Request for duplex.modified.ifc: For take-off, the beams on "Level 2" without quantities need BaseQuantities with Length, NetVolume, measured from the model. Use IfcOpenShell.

First a look at what the model holds.

```python
import ifcopenshell
import ifcopenshell.util.element
import ifcopenshell.util.unit

model = ifcopenshell.open("duplex.modified.ifc")
print(model.schema)
for unit_type in ("LENGTHUNIT", "AREAUNIT", "VOLUMEUNIT"):
    print(unit_type, ifcopenshell.util.unit.calculate_unit_scale(model, unit_type))
storey = next(s for s in model.by_type("IfcBuildingStorey") if s.Name == "Level 2")
beams = [e for e in ifcopenshell.util.element.get_decomposition(storey) if e.is_a("IfcBeam")]
for e in sorted(beams, key=lambda e: e.id()):
    print(e.id(), e.is_a(), e.Name, list(ifcopenshell.util.element.get_psets(e, qtos_only=True)), sep=" | ")
```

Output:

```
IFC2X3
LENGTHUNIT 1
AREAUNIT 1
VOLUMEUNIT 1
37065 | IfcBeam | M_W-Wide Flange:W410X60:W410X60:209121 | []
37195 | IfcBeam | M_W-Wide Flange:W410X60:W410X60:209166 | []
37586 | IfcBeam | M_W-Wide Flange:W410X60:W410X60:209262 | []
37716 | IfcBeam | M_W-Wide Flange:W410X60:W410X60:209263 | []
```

```python
import ifcopenshell
import ifcopenshell.api.pset
import ifcopenshell.geom
import ifcopenshell.util.element
import ifcopenshell.util.shape
import ifcopenshell.util.unit

model = ifcopenshell.open("duplex.modified.ifc")
unit_scale = ifcopenshell.util.unit.calculate_unit_scale(model)
volume_scale = ifcopenshell.util.unit.calculate_unit_scale(model, "VOLUMEUNIT")
settings = ifcopenshell.geom.settings()

storey = next(s for s in model.by_type("IfcBuildingStorey") if s.Name == "Level 2")
beams = [e for e in ifcopenshell.util.element.get_decomposition(storey) if e.is_a("IfcBeam")]

for e in sorted(beams, key=lambda e: e.id()):
    if ifcopenshell.util.element.get_psets(e, qtos_only=True, should_inherit=False):
        continue
    # Geometry comes back in metres, in the element's own axes.
    shape = ifcopenshell.geom.create_shape(settings, e)
    values = {
        "Length": ifcopenshell.util.shape.get_max_xyz(shape.geometry) / unit_scale,
        "NetVolume": ifcopenshell.util.shape.get_volume(shape.geometry) / volume_scale,
    }
    qto = ifcopenshell.api.pset.add_qto(model, product=e, name="BaseQuantities")
    ifcopenshell.api.pset.edit_qto(model, qto=qto, properties=values)
    print(e.id(), {k: round(v, 3) for k, v in values.items()})

model.write("duplex.modified_updated.ifc")
```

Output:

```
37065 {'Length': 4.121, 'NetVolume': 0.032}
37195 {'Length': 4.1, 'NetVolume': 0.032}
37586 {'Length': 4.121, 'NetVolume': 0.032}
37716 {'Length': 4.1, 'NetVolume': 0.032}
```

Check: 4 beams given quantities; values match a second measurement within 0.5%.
